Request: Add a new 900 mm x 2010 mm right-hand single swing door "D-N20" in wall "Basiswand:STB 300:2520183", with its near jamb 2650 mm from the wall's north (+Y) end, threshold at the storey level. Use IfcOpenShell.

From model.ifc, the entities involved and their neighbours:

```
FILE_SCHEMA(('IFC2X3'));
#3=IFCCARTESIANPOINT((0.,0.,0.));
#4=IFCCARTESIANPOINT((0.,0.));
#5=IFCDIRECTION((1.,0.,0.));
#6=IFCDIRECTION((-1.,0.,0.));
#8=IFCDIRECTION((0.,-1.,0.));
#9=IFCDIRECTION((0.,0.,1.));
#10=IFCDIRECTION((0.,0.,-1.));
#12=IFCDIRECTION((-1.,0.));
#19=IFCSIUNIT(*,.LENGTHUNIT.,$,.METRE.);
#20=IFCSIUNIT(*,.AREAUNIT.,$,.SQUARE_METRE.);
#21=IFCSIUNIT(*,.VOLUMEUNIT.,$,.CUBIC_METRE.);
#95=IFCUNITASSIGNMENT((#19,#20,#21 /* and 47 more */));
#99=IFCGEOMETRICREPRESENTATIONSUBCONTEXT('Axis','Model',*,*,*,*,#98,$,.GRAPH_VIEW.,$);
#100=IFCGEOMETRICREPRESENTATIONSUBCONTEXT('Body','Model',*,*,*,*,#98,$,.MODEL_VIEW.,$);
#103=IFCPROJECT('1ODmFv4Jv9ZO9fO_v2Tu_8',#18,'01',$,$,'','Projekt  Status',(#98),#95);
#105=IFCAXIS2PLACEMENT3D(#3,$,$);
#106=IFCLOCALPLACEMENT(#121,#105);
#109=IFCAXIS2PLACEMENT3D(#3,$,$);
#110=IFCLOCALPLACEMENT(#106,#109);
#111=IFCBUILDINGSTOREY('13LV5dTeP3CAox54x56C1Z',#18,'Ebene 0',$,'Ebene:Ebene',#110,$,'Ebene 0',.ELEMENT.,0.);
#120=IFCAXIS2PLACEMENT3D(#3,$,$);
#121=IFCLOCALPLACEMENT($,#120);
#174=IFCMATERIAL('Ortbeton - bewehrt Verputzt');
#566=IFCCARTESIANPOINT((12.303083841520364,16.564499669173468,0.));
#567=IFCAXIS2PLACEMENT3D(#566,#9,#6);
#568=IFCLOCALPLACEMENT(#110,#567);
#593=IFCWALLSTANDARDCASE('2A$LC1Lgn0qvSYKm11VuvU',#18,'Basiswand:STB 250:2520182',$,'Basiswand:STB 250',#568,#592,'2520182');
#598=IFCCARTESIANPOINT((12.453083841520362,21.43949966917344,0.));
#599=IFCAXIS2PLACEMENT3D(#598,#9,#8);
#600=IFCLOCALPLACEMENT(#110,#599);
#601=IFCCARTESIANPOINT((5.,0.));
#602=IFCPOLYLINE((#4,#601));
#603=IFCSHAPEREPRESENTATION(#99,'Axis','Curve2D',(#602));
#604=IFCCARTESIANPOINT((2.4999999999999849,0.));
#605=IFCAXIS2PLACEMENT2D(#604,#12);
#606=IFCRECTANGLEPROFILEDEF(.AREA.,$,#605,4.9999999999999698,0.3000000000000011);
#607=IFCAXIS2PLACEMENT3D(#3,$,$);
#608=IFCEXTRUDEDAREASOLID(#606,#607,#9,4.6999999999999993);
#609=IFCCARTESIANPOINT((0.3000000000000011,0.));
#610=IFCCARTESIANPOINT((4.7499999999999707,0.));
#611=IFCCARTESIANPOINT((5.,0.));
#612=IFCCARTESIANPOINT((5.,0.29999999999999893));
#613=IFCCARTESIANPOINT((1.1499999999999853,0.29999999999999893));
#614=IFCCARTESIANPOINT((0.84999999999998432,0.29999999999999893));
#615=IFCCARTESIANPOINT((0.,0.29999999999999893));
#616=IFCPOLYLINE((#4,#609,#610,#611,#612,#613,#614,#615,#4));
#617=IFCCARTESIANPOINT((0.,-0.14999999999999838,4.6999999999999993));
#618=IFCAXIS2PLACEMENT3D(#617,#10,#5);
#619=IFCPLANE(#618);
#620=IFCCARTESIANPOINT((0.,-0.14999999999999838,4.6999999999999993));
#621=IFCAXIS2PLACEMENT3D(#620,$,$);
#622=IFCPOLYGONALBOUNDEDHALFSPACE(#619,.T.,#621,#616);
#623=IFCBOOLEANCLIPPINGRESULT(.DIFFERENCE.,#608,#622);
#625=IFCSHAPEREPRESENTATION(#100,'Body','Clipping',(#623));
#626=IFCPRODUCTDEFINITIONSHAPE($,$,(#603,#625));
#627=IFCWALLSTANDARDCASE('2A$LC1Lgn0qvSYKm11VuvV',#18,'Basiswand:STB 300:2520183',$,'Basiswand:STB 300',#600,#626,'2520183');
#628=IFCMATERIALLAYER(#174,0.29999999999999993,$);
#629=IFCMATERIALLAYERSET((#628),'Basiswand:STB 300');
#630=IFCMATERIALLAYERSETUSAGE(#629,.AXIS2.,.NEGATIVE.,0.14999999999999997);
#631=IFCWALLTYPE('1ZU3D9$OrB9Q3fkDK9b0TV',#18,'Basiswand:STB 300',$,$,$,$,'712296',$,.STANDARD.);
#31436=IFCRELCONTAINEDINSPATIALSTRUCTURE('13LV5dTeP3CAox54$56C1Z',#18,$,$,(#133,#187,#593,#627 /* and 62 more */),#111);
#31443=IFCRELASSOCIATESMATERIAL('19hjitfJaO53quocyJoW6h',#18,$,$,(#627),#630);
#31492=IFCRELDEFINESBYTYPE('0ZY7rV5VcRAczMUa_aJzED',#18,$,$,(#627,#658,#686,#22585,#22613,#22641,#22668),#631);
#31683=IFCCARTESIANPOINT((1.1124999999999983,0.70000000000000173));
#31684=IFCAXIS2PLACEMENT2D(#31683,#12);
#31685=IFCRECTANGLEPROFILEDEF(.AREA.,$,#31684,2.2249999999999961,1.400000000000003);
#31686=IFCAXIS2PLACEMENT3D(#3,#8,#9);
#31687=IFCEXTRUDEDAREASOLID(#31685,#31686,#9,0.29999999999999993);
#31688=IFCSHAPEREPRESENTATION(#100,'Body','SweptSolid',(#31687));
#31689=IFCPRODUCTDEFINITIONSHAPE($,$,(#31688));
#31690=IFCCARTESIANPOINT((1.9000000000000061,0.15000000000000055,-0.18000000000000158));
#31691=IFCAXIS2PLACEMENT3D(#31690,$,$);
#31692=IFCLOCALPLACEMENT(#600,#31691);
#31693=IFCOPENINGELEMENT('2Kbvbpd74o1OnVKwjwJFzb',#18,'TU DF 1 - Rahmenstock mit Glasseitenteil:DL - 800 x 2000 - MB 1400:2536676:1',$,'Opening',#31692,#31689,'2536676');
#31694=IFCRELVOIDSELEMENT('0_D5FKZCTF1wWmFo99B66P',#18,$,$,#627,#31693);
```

```python
import numpy as np
import ifcopenshell
import ifcopenshell.api.feature
import ifcopenshell.api.geometry
import ifcopenshell.api.root
import ifcopenshell.api.spatial
import ifcopenshell.api.type
import ifcopenshell.geom
import ifcopenshell.util.element
import ifcopenshell.util.placement
import ifcopenshell.util.representation
import ifcopenshell.util.shape
import ifcopenshell.util.unit

model = ifcopenshell.open("model.ifc")
unit_scale = ifcopenshell.util.unit.calculate_unit_scale(model)
settings = ifcopenshell.geom.settings()


def volume(element):
    """Net volume in cubic metres, openings subtracted."""
    shape = ifcopenshell.geom.create_shape(settings, element)
    return ifcopenshell.util.shape.get_volume(shape.geometry)


wall = model.by_id(627)
storey = ifcopenshell.util.element.get_container(wall, ifc_class="IfcBuildingStorey")
context = ifcopenshell.util.representation.get_context(model, "Model", "Body", "MODEL_VIEW")
before = volume(wall)

width, height, from_end, sill = 0.9, 2.01, 2.65, 0.0  # metres

# The wall runs along its own X axis, and the end named is its -X end.
wall_shape = ifcopenshell.geom.create_shape(settings, wall)
x, y, z = ifcopenshell.util.shape.get_vertices(wall_shape.geometry).T
start = x.min() + from_end
face, thickness = float(y.min()), float(y.max() - y.min())
wall_matrix = ifcopenshell.util.placement.get_local_placement(wall.ObjectPlacement)
level = ifcopenshell.util.placement.get_local_placement(storey.ObjectPlacement)[2, 3]


def in_wall(x, y):
    """Placement at x, y metres in the wall's axes, at sill height."""
    matrix = wall_matrix.copy()
    matrix[:, 3] = wall_matrix @ np.array([x / unit_scale, y / unit_scale, 0.0, 1.0])
    matrix[2, 3] = level + sill / unit_scale
    return matrix


# Opening: a box that overshoots both wall faces by 50 mm.
opening = ifcopenshell.api.root.create_entity(model, ifc_class="IfcOpeningElement")
box = ifcopenshell.api.geometry.add_wall_representation(
    model, context=context, length=width, height=height, thickness=thickness + 0.1
)
ifcopenshell.api.geometry.assign_representation(model, product=opening, representation=box)
ifcopenshell.api.geometry.edit_object_placement(model, product=opening, matrix=in_wall(start, face - 0.05), is_si=False)
ifcopenshell.api.feature.add_feature(model, feature=opening, element=wall)

door = ifcopenshell.api.root.create_entity(model, ifc_class="IfcDoor", name="D-N20")
door.OverallWidth, door.OverallHeight = width / unit_scale, height / unit_scale
body = ifcopenshell.api.geometry.add_door_representation(
    model,
    context=context,
    overall_width=door.OverallWidth,
    overall_height=door.OverallHeight,
    operation_type="SINGLE_SWING_RIGHT",
    lining_properties={"LiningDepth": thickness / unit_scale, "ThresholdDepth": thickness / unit_scale},
)
ifcopenshell.api.geometry.assign_representation(model, product=door, representation=body)
ifcopenshell.api.spatial.assign_container(model, products=[door], relating_structure=storey)
fills = ifcopenshell.api.feature.add_filling(model, opening=opening, element=door)
fills.OwnerHistory = door.OwnerHistory  # required in IFC2X3

# IFC2X3 keeps the operation on the door style.
style = ifcopenshell.api.root.create_entity(model, ifc_class="IfcDoorStyle", name="D-N20")
style.OperationType, style.ConstructionType = "SINGLE_SWING_RIGHT", "NOTDEFINED"
style.ParameterTakesPrecedence = style.Sizeable = False
ifcopenshell.api.type.assign_type(model, related_objects=[door], relating_type=style)

# The lining spans the wall, so the door starts at the wall face.
ifcopenshell.api.geometry.edit_object_placement(model, product=door, matrix=in_wall(start, face), is_si=False)

after = volume(wall)

print(f"wall volume {before:.3f} -> {after:.3f} m3")

model.write("model_updated.ifc")
```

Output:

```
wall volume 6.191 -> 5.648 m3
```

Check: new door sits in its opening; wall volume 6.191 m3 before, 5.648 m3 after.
